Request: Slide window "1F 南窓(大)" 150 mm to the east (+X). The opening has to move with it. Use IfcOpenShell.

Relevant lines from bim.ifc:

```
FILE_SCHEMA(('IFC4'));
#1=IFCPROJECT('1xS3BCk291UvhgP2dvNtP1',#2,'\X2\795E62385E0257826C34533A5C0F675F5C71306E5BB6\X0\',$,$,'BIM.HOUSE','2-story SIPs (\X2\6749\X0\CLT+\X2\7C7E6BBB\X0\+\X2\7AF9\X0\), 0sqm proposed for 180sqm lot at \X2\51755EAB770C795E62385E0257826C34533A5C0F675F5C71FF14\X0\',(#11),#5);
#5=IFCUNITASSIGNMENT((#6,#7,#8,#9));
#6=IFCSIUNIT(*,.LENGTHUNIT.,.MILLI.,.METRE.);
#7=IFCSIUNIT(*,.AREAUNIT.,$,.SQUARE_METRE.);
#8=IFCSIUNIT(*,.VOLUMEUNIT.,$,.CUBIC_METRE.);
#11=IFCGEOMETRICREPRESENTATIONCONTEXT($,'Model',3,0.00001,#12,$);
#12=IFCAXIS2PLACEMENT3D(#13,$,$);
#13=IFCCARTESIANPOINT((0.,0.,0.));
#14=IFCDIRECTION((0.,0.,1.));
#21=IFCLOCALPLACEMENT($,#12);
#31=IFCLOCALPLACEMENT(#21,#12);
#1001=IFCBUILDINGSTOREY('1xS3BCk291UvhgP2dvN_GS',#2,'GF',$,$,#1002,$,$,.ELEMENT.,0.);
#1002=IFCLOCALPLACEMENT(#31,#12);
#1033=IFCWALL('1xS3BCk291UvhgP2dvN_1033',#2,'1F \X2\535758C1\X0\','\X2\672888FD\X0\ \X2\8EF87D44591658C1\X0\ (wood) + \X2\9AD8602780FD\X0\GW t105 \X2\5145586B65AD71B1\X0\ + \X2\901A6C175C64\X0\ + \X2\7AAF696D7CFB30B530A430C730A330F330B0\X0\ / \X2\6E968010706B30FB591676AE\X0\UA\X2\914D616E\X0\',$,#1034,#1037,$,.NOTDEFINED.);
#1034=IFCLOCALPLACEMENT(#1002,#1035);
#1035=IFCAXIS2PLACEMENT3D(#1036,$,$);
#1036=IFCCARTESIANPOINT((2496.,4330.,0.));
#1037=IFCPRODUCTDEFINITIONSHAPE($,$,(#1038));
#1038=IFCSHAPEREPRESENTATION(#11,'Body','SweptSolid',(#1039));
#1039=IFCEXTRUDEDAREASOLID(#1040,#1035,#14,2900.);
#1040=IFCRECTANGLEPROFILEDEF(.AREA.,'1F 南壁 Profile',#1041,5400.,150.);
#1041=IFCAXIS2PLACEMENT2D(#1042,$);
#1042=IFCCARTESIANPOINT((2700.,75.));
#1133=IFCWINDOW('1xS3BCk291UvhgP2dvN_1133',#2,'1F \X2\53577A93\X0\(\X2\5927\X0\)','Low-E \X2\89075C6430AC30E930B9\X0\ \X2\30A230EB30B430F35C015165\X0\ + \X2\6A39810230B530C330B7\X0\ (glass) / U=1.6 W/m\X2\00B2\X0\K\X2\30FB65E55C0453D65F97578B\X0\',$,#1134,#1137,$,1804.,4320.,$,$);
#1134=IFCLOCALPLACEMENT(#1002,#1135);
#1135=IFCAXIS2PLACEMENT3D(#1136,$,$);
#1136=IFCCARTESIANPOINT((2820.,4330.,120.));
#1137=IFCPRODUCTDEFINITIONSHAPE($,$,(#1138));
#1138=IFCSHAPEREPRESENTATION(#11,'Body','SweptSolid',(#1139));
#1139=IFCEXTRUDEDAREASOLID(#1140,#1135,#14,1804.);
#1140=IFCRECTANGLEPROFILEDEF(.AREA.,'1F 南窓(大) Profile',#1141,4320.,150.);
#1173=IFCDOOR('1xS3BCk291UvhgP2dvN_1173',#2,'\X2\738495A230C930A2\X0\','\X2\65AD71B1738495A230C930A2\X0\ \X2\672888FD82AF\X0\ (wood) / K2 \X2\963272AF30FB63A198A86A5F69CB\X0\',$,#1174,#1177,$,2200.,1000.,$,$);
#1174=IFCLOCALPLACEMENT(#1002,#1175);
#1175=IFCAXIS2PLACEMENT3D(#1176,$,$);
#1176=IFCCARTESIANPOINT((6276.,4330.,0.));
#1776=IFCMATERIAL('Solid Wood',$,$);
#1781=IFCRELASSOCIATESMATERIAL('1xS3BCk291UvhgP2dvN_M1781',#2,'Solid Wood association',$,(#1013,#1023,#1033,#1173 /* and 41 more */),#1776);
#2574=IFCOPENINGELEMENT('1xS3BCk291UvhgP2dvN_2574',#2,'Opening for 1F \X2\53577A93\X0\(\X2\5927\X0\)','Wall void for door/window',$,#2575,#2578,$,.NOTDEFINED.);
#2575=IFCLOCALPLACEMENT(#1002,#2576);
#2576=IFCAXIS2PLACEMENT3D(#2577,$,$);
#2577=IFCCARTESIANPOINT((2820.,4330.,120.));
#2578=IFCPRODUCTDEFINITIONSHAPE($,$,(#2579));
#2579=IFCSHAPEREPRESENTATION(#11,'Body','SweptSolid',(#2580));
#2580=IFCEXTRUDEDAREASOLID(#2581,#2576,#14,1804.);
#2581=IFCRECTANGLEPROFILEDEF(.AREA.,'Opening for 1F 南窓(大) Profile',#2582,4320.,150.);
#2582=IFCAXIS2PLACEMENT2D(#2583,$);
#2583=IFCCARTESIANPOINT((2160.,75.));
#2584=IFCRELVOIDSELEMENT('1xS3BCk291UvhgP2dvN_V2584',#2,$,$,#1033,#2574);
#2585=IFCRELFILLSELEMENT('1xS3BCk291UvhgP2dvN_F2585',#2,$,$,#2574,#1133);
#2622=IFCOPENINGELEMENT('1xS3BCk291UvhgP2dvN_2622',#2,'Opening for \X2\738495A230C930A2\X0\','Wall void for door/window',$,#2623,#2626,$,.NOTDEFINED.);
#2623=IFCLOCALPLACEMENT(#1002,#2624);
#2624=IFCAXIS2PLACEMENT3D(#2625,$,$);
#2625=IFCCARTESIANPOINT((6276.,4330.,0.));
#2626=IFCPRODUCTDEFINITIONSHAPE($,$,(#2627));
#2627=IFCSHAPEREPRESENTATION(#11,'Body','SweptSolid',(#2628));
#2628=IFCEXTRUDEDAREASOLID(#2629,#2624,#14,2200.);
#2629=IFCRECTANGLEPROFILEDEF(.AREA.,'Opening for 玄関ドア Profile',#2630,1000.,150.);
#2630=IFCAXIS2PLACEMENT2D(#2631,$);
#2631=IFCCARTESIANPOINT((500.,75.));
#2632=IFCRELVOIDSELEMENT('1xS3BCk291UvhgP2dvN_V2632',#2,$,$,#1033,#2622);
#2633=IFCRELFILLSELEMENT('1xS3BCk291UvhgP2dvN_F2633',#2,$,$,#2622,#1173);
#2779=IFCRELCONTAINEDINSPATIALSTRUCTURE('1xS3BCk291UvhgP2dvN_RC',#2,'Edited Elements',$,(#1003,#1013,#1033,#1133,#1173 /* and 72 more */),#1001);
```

```python
import ifcopenshell
import ifcopenshell.api.geometry
import ifcopenshell.util.placement

model = ifcopenshell.open("bim.ifc")

window = model.by_guid("1xS3BCk291UvhgP2dvN_1133")
opening = window.FillsVoids[0].RelatingOpeningElement
wall = opening.VoidsElements[0].RelatingBuildingElement

wall_matrix = ifcopenshell.util.placement.get_local_placement(wall.ObjectPlacement)
shift = wall_matrix[:3, 0] * 150.0
before = ifcopenshell.util.placement.get_local_placement(window.ObjectPlacement)[:3, 3].copy()

# The window is not placed relative to its opening, so move both.
for product in (opening, window):
    matrix = ifcopenshell.util.placement.get_local_placement(product.ObjectPlacement)
    matrix[:3, 3] += shift
    ifcopenshell.api.geometry.edit_object_placement(model, product=product, matrix=matrix, is_si=False)

after = ifcopenshell.util.placement.get_local_placement(window.ObjectPlacement)[:3, 3]
print("window moved by", (after - before).round(3) + 0.0)

model.write("bim-out.ifc")
```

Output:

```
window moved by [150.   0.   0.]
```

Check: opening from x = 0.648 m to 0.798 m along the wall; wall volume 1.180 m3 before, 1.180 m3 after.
